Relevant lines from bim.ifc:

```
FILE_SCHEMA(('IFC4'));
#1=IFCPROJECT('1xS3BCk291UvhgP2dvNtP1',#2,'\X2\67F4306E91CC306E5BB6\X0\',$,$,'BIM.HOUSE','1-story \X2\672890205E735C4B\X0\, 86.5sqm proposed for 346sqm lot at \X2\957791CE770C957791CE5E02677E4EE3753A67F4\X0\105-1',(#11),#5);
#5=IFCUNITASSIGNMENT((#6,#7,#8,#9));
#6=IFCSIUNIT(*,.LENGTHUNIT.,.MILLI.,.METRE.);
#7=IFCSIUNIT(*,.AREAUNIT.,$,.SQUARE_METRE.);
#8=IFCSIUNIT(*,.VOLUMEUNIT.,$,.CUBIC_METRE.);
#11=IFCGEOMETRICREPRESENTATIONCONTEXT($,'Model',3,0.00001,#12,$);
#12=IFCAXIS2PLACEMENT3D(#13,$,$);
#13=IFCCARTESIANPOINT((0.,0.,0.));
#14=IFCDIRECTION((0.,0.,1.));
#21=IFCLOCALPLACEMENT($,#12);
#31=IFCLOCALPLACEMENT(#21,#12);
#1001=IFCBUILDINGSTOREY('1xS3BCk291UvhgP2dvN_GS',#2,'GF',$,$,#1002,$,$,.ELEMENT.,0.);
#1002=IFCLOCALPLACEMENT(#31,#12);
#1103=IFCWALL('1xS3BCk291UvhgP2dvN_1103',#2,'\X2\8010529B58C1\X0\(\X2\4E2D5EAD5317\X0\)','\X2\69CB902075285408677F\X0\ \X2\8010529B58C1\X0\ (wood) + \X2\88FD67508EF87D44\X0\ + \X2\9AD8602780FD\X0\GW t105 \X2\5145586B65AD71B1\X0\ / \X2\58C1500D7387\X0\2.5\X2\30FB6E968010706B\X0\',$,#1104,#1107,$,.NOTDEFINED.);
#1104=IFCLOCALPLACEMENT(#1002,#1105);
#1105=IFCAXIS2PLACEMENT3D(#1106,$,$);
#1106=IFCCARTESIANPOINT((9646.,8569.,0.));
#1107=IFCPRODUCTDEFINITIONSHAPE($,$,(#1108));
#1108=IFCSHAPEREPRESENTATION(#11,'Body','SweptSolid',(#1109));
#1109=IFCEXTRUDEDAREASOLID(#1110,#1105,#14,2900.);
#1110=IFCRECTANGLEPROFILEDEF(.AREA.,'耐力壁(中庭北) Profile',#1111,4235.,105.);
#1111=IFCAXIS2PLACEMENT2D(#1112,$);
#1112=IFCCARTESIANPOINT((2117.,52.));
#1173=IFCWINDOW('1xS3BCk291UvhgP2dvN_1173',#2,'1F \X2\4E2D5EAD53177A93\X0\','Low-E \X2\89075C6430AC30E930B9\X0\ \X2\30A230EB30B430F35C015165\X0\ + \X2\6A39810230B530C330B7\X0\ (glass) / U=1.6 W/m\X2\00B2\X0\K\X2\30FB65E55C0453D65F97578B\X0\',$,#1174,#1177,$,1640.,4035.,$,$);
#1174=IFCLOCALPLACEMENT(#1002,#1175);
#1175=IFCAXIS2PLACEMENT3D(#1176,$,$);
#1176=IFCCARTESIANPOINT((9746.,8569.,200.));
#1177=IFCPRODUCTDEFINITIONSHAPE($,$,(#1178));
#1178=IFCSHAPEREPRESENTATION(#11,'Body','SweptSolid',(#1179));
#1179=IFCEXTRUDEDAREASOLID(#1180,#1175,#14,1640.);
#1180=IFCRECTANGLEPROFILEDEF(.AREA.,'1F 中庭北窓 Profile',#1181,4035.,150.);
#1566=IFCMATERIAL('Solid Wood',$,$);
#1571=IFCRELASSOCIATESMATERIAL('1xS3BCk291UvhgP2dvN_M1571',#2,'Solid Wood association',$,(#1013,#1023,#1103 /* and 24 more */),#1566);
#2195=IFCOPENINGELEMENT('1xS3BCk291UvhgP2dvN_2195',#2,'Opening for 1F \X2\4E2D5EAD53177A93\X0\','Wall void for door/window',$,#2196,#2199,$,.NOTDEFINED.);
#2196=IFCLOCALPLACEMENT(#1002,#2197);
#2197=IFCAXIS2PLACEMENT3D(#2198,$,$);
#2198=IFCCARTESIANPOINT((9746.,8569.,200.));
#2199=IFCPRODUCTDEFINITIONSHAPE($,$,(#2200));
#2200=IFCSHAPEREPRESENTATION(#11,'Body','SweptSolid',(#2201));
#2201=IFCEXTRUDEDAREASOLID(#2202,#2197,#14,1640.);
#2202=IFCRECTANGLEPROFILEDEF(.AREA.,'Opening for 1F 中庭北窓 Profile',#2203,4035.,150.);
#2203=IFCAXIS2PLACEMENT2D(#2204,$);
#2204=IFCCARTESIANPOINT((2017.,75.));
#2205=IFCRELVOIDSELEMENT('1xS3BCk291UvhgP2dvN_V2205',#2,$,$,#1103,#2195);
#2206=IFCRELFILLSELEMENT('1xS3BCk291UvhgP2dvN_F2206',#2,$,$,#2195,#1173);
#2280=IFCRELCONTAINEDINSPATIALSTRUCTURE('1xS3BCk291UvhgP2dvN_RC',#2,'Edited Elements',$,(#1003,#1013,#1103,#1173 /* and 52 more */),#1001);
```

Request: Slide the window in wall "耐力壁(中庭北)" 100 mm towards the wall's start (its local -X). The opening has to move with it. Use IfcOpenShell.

```python
import ifcopenshell
import ifcopenshell.api.geometry
import ifcopenshell.util.placement
import ifcopenshell.util.unit

model = ifcopenshell.open("bim.ifc")
unit_scale = ifcopenshell.util.unit.calculate_unit_scale(model)

window = model.by_id(1173)
opening = window.FillsVoids[0].RelatingOpeningElement
wall = opening.VoidsElements[0].RelatingBuildingElement

wall_matrix = ifcopenshell.util.placement.get_local_placement(wall.ObjectPlacement)
shift = wall_matrix[:3, 0] * -0.1 / unit_scale
before = ifcopenshell.util.placement.get_local_placement(window.ObjectPlacement)[:3, 3].copy()

# The window is not placed relative to its opening, so move both.
for product in (opening, window):
    matrix = ifcopenshell.util.placement.get_local_placement(product.ObjectPlacement)
    matrix[:3, 3] += shift
    ifcopenshell.api.geometry.edit_object_placement(model, product=product, matrix=matrix, is_si=False)

after = ifcopenshell.util.placement.get_local_placement(window.ObjectPlacement)[:3, 3]
print("window moved by", (after - before).round(3) + 0.0)

model.write("bim-out.ifc")
```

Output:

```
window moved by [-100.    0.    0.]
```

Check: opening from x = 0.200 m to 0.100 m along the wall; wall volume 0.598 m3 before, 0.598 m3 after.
